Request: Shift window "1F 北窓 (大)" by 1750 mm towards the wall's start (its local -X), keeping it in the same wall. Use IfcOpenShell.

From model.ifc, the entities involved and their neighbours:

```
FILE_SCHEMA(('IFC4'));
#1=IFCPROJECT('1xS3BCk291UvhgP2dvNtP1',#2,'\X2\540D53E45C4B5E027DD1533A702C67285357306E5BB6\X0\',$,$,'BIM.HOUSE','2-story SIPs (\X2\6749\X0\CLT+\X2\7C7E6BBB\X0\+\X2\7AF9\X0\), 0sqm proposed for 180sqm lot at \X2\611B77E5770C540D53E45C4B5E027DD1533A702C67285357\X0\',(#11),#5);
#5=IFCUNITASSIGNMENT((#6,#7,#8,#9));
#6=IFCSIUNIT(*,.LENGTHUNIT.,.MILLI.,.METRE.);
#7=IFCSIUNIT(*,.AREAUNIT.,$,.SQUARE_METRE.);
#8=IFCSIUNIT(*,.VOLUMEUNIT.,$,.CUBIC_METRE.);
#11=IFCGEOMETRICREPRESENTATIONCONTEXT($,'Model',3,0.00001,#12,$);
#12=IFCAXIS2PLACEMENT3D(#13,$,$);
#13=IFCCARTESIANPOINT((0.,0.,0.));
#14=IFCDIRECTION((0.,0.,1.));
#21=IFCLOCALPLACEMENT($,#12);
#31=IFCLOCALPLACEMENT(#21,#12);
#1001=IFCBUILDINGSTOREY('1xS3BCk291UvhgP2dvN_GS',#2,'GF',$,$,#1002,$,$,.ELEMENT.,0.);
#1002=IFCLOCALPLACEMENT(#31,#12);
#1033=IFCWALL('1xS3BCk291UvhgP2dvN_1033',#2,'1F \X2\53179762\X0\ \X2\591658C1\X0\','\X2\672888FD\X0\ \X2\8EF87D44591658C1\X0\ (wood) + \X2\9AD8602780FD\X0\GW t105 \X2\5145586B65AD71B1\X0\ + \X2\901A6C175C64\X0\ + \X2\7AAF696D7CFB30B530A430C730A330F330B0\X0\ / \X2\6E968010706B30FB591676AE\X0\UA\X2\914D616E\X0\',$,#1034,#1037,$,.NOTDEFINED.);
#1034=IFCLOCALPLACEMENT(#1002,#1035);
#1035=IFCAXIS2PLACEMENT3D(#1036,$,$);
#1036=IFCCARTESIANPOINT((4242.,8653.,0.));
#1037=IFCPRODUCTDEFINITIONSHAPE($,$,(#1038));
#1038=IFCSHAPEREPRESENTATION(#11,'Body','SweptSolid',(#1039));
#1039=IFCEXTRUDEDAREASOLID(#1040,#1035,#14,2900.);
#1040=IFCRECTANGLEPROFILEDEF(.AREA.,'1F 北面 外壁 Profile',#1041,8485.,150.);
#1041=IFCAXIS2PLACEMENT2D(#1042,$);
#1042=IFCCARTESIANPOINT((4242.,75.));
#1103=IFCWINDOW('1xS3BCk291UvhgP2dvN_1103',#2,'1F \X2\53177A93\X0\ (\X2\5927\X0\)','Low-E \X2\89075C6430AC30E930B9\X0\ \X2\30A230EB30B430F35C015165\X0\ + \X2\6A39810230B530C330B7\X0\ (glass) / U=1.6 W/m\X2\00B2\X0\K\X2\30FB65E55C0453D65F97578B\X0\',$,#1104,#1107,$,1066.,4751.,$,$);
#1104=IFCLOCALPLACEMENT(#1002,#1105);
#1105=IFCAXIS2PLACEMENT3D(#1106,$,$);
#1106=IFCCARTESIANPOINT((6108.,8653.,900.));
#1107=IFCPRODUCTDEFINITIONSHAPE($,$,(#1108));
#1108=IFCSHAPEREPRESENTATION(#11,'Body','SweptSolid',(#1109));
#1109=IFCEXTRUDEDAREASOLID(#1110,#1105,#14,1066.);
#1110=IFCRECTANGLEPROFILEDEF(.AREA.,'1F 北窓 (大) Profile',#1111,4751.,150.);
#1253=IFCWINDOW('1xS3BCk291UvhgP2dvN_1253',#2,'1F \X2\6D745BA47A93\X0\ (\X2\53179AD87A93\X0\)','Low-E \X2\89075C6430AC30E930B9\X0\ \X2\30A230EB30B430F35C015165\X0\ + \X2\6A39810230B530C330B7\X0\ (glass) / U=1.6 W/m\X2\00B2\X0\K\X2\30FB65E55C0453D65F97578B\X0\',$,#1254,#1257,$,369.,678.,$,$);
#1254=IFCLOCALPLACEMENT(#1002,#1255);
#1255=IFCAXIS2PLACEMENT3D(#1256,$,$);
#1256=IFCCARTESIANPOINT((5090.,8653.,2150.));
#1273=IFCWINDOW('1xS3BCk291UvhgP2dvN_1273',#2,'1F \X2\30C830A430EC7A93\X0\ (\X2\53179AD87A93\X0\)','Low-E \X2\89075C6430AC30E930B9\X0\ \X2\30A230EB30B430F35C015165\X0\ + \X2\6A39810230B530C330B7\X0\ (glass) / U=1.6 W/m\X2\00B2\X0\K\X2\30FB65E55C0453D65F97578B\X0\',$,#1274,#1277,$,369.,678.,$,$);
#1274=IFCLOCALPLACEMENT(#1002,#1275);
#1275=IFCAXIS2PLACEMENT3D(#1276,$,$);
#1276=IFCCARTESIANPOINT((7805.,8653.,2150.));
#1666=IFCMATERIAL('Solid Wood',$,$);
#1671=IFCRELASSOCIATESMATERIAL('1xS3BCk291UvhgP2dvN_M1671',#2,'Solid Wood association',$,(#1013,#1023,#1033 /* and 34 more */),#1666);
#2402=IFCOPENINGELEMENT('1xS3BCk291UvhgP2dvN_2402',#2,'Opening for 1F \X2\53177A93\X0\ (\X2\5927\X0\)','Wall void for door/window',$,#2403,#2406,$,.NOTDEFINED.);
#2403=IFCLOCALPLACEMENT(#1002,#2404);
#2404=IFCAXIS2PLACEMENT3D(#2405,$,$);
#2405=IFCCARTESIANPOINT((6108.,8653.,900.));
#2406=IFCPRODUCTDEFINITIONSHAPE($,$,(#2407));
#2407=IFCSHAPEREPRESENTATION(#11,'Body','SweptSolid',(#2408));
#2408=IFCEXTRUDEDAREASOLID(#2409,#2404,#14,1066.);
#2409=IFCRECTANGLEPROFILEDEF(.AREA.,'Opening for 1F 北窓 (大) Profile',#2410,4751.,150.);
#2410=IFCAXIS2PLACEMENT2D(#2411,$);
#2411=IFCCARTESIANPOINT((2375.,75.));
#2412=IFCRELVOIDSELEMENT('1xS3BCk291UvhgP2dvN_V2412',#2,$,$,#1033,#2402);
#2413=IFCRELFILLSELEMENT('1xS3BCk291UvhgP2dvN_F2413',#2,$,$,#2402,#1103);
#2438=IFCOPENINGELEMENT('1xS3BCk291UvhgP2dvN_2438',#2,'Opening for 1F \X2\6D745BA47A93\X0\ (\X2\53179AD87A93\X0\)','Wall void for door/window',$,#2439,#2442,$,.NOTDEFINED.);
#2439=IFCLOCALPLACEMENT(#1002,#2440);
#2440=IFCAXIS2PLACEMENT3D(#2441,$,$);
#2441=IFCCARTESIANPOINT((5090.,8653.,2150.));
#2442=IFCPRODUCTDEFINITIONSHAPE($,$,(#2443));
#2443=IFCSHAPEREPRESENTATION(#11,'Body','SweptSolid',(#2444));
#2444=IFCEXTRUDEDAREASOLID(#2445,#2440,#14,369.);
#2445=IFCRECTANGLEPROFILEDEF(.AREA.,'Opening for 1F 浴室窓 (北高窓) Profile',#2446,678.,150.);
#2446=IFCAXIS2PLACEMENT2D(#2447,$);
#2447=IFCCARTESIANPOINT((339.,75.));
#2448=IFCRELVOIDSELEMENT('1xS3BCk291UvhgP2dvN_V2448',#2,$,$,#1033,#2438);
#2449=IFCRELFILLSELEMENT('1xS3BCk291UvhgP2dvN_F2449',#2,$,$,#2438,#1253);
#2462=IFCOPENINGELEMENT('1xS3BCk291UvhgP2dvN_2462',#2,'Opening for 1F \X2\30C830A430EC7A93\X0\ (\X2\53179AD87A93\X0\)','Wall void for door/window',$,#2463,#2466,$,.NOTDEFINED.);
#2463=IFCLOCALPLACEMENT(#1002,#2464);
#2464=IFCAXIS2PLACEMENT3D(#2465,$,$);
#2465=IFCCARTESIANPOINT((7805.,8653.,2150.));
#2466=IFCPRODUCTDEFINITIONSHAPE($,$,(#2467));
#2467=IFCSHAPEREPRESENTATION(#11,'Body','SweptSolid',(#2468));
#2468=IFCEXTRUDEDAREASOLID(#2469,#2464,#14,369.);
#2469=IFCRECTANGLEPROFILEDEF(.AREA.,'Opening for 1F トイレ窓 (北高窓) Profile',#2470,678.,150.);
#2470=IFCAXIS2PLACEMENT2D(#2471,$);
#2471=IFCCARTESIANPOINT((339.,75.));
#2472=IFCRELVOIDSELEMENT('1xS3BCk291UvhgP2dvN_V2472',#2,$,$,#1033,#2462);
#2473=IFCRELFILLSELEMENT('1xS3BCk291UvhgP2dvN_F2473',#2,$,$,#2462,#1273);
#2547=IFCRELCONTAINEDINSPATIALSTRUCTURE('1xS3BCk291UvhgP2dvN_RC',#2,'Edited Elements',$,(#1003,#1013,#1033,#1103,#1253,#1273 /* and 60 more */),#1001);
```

```python
import ifcopenshell
import ifcopenshell.api.geometry
import ifcopenshell.util.placement

model = ifcopenshell.open("model.ifc")

window = model.by_guid("1xS3BCk291UvhgP2dvN_1103")
opening = window.FillsVoids[0].RelatingOpeningElement
wall = opening.VoidsElements[0].RelatingBuildingElement

wall_matrix = ifcopenshell.util.placement.get_local_placement(wall.ObjectPlacement)
shift = wall_matrix[:3, 0] * -1750.0
before = ifcopenshell.util.placement.get_local_placement(window.ObjectPlacement)[:3, 3].copy()

# The window is not placed relative to its opening, so move both.
for product in (opening, window):
    matrix = ifcopenshell.util.placement.get_local_placement(product.ObjectPlacement)
    matrix[:3, 3] += shift
    ifcopenshell.api.geometry.edit_object_placement(model, product=product, matrix=matrix, is_si=False)

after = ifcopenshell.util.placement.get_local_placement(window.ObjectPlacement)[:3, 3]
print("window moved by", (after - before).round(3) + 0.0)

model.write("model_v2.ifc")
```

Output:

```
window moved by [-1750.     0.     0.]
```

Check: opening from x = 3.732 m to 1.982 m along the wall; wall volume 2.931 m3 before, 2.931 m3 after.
